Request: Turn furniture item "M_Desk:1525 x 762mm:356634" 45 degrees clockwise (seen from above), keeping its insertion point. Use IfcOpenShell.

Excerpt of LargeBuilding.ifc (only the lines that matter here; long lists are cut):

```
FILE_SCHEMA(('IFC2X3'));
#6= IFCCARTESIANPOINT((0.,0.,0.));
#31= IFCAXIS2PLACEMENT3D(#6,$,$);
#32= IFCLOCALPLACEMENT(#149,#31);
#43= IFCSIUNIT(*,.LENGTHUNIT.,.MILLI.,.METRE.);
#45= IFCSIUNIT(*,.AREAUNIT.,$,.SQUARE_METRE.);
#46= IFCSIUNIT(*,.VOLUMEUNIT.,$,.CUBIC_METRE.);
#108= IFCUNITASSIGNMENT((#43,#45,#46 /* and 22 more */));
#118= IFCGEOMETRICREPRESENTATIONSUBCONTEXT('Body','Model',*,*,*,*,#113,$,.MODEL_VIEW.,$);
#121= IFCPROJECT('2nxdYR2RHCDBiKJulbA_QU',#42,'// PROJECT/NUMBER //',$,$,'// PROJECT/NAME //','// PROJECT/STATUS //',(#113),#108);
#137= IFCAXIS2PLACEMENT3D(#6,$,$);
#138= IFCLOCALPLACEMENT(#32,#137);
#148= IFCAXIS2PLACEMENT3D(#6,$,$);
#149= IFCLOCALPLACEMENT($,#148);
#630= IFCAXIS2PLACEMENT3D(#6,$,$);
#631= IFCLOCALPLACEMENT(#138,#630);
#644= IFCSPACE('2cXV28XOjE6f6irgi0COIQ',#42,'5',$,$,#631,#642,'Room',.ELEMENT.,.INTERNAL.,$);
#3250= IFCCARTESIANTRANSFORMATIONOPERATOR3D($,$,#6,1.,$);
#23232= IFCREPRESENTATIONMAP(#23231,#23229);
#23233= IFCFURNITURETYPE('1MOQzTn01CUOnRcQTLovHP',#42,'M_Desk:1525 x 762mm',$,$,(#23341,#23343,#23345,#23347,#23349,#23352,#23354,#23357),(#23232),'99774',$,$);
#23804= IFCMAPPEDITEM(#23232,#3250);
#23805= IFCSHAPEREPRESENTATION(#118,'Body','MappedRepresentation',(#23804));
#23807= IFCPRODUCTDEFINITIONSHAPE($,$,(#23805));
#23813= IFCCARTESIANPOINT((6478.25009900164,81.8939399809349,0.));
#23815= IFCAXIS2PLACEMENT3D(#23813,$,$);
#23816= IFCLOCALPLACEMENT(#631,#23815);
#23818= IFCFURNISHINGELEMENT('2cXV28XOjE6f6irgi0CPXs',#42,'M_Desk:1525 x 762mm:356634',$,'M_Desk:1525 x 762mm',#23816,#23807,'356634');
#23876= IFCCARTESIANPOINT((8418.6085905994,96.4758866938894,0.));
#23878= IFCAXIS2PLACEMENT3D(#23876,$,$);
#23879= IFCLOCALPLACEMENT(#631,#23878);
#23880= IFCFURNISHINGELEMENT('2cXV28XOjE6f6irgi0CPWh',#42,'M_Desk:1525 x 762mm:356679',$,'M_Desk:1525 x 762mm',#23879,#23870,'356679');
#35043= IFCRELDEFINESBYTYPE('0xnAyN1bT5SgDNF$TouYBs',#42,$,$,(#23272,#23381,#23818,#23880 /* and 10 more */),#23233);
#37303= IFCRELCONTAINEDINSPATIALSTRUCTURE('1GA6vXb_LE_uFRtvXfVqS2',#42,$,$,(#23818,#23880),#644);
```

```python
import ifcopenshell
import ifcopenshell.api.geometry
import ifcopenshell.util.placement

model = ifcopenshell.open("LargeBuilding.ifc")

item = model.by_guid("2cXV28XOjE6f6irgi0CPXs")
matrix = ifcopenshell.util.placement.get_local_placement(item.ObjectPlacement)
matrix = matrix @ ifcopenshell.util.placement.rotation(-45, "Z")
ifcopenshell.api.geometry.edit_object_placement(model, product=item, matrix=matrix, is_si=False)

print(ifcopenshell.util.placement.get_local_placement(item.ObjectPlacement).round(3) + 0.0)

model.write("LargeBuilding_edited.ifc")
```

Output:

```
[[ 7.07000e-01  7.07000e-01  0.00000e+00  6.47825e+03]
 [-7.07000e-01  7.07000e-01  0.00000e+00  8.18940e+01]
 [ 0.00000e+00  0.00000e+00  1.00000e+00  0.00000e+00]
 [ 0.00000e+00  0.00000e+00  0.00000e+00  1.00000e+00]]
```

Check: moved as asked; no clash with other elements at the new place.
